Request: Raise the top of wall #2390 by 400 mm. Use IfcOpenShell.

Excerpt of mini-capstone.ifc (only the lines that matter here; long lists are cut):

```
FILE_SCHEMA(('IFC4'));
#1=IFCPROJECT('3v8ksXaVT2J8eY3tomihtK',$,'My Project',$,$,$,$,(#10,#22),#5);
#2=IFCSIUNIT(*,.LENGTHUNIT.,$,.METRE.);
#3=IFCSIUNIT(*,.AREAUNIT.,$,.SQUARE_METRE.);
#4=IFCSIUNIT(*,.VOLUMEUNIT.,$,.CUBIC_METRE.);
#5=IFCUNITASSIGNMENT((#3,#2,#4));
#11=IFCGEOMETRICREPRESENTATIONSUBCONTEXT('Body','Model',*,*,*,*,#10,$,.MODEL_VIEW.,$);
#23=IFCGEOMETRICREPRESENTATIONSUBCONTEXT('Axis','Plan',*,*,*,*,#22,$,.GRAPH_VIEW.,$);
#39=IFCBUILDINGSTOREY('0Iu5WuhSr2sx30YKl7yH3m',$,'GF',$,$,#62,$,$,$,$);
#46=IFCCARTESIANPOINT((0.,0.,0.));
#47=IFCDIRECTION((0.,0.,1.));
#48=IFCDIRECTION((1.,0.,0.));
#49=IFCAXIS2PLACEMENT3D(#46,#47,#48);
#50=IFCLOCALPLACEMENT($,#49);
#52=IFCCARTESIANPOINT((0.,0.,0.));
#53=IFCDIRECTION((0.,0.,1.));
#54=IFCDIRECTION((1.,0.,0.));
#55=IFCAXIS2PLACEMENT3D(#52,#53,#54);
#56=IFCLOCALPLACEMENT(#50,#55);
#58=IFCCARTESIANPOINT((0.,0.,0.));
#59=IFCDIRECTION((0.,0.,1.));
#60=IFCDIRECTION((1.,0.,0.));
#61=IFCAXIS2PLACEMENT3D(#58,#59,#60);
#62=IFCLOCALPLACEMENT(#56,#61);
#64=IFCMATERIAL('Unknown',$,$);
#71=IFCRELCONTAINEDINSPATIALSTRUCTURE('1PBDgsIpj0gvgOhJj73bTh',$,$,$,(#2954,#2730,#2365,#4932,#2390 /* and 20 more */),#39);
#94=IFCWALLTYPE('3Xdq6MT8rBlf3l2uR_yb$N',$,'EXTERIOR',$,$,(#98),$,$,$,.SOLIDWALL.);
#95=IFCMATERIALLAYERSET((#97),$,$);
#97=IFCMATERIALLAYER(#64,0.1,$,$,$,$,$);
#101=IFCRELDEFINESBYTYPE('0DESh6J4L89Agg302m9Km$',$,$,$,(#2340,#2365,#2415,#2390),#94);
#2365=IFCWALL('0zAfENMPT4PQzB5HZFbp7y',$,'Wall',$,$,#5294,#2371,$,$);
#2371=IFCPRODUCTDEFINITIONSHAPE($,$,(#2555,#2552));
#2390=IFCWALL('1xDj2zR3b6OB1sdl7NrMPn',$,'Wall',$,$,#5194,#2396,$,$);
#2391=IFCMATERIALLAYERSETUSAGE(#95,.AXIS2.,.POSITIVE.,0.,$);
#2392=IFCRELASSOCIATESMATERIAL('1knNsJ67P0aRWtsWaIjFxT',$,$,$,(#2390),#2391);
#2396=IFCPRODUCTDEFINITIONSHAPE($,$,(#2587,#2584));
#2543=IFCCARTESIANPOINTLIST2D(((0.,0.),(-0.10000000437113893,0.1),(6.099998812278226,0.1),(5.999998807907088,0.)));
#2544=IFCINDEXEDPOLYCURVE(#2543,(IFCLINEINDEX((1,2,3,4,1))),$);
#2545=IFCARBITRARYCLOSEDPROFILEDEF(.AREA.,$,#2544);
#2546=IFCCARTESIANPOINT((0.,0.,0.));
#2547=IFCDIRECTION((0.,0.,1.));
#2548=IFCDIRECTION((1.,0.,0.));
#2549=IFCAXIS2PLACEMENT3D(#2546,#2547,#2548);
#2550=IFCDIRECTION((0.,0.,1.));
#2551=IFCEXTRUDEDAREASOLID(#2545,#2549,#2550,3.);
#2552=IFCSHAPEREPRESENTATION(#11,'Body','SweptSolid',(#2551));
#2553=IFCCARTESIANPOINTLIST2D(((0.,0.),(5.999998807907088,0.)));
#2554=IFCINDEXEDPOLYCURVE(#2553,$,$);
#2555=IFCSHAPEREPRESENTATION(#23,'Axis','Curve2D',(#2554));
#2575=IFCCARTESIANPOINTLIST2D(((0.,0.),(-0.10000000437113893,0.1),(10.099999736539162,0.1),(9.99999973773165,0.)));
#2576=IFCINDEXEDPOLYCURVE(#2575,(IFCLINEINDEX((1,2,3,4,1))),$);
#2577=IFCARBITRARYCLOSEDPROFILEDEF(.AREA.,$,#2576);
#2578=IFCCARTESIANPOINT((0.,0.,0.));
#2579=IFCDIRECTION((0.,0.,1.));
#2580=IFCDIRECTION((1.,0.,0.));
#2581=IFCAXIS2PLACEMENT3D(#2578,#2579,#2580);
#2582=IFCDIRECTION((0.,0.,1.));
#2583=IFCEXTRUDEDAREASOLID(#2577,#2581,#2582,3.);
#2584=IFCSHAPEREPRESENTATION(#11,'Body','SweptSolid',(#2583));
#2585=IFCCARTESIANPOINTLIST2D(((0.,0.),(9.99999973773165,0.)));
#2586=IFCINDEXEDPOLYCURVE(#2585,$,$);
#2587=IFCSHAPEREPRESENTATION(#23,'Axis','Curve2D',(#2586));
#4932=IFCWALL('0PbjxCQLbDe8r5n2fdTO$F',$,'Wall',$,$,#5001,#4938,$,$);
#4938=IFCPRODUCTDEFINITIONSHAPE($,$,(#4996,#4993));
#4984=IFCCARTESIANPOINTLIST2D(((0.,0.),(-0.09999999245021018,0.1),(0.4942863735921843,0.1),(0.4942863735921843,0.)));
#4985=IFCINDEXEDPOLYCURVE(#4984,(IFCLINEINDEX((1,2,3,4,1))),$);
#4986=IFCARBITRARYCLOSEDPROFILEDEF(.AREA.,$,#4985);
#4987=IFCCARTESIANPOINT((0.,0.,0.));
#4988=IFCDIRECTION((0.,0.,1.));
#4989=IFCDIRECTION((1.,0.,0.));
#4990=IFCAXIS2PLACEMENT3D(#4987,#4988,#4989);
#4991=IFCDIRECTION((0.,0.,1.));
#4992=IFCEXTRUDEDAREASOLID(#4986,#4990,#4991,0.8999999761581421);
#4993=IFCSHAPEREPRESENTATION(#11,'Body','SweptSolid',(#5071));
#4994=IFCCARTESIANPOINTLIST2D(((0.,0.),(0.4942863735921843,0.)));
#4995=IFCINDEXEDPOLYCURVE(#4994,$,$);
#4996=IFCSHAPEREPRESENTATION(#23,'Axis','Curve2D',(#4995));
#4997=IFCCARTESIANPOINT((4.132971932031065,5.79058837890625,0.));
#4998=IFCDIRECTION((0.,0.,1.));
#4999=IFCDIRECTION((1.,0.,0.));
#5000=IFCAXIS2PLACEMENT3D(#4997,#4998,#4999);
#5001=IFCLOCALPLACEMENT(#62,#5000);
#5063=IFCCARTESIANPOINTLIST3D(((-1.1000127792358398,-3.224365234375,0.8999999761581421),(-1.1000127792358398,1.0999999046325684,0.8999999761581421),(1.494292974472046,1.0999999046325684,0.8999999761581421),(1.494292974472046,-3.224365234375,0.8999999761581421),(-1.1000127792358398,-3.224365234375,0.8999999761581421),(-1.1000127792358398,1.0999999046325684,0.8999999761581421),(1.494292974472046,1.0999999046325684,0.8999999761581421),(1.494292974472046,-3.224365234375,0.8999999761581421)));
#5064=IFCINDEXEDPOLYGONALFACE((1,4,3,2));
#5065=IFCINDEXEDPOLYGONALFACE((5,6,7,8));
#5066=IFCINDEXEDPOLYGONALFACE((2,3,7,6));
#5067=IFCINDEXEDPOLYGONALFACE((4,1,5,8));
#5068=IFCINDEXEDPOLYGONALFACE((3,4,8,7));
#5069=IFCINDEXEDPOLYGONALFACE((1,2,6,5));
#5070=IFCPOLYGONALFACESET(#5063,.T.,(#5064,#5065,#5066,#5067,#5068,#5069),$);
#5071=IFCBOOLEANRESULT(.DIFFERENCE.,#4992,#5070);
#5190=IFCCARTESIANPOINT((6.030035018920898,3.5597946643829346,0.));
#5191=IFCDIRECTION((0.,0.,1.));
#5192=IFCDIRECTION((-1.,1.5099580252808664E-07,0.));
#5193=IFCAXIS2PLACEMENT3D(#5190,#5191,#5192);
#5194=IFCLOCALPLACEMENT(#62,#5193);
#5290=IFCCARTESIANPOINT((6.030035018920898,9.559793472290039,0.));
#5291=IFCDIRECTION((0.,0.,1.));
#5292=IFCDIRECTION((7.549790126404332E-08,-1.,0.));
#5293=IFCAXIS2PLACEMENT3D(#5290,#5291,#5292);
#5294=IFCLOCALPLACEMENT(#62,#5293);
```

```python
import ifcopenshell
import ifcopenshell.geom
import ifcopenshell.util.representation
import ifcopenshell.util.shape
import ifcopenshell.util.unit

model = ifcopenshell.open("mini-capstone.ifc")
unit_scale = ifcopenshell.util.unit.calculate_unit_scale(model)
settings = ifcopenshell.geom.settings()


def volume(element):
    """Net volume in cubic metres, openings subtracted."""
    shape = ifcopenshell.geom.create_shape(settings, element)
    return ifcopenshell.util.shape.get_volume(shape.geometry)


wall = model.by_guid("1xDj2zR3b6OB1sdl7NrMPn")
before = volume(wall)

body = ifcopenshell.util.representation.get_representation(wall, "Model", "Body")
solid = body.Items[0]
old_height = solid.Depth
solid.Depth += 0.4 / unit_scale
after = volume(wall)

print(f"height {old_height:g} -> {solid.Depth:g}, volume {before:.3f} -> {after:.3f} m3")

model.write("mini-capstone_v2.ifc")
```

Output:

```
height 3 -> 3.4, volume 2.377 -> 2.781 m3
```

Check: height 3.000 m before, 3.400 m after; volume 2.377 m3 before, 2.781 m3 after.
